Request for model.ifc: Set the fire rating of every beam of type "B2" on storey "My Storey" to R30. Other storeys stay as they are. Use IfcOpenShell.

First a look at what the model holds.

```python
import ifcopenshell
import ifcopenshell.util.element

model = ifcopenshell.open("model.ifc")
print(model.schema)
storey = next(s for s in model.by_type("IfcBuildingStorey") if s.Name == "My Storey")
beams = [e for e in ifcopenshell.util.element.get_decomposition(storey) if e.is_a("IfcBeam")]
seen = {}
for e in beams:
    element_type = ifcopenshell.util.element.get_type(e)
    key = (element_type.Name if element_type != e and element_type else None, ifcopenshell.util.element.get_pset(e, "Pset_BeamCommon", "FireRating"))
    seen[key] = seen.get(key, 0) + 1
for (name, value), count in sorted(seen.items(), key=str):
    print(count, "x", name, "|", value)
```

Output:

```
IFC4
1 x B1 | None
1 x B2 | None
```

```python
import ifcopenshell
import ifcopenshell.api.pset
import ifcopenshell.util.element

model = ifcopenshell.open("model.ifc")

storey = next(s for s in model.by_type("IfcBuildingStorey") if s.Name == "My Storey")
beams = [e for e in ifcopenshell.util.element.get_decomposition(storey) if e.is_a("IfcBeam")]

count = 0
for e in beams:
    element_type = ifcopenshell.util.element.get_type(e)
    if element_type in (None, e) or element_type.Name != "B2":
        continue
    # add_pset returns the element's existing set when there is one.
    pset = ifcopenshell.api.pset.add_pset(model, product=e, name="Pset_BeamCommon")
    ifcopenshell.api.pset.edit_pset(model, pset=pset, properties={"FireRating": "R30"})
    count += 1

print(count, "beams updated")

model.write("model_updated.ifc")
```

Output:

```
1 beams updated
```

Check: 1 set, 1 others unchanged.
